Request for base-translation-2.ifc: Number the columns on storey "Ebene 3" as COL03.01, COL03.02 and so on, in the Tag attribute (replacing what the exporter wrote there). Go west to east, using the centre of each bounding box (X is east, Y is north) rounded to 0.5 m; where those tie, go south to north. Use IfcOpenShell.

First a look at what the model holds.

```python
import ifcopenshell
import ifcopenshell.util.element
import ifcopenshell.util.placement

model = ifcopenshell.open("base-translation-2.ifc")
print(model.schema)
storey = next(s for s in model.by_type("IfcBuildingStorey") if s.Name == "Ebene 3")
columns = [e for e in ifcopenshell.util.element.get_decomposition(storey) if e.is_a("IfcColumn")]
for e in sorted(columns, key=lambda e: e.id()):
    origin = ifcopenshell.util.placement.get_local_placement(e.ObjectPlacement)[:3, 3]
    print(e.id(), e.Tag, e.Name, origin.round(2) + 0.0, sep=" | ")
```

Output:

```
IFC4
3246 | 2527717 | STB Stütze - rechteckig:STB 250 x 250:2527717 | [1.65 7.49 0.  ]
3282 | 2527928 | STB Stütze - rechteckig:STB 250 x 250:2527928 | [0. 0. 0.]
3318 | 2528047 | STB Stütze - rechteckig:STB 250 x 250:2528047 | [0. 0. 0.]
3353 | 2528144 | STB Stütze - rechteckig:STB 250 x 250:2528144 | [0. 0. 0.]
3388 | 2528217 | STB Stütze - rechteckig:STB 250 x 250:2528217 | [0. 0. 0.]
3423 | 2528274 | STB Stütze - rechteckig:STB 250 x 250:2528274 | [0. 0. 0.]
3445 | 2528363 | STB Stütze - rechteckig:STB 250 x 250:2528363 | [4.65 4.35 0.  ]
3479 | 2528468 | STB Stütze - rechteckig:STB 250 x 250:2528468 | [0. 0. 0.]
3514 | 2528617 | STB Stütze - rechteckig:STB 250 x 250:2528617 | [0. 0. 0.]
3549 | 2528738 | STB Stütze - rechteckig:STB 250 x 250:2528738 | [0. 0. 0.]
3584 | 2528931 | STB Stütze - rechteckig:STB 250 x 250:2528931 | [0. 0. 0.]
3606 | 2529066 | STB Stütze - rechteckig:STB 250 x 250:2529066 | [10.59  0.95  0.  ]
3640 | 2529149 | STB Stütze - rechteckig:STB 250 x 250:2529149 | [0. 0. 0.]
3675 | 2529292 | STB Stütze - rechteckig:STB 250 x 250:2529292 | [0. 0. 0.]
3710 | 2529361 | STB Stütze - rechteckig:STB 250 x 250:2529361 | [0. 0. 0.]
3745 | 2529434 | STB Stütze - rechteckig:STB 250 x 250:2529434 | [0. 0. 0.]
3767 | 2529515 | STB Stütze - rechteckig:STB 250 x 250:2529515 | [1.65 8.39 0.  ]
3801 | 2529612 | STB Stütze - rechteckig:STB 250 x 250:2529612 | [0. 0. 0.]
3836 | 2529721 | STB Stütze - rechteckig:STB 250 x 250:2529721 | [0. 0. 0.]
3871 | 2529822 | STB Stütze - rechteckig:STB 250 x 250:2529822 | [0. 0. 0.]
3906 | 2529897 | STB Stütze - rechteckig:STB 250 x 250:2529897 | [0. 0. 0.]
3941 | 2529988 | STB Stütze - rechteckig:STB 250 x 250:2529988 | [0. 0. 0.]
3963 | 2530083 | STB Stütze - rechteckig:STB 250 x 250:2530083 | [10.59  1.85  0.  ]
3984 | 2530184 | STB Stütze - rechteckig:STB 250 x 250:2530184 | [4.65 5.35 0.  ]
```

```python
import ifcopenshell
import ifcopenshell.geom
import ifcopenshell.util.element
import ifcopenshell.util.shape

model = ifcopenshell.open("base-translation-2.ifc")
settings = ifcopenshell.geom.settings()
settings.set("use-world-coords", True)


def centre(element):
    shape = ifcopenshell.geom.create_shape(settings, element)
    return ifcopenshell.util.shape.get_bbox_centroid(shape.geometry)


storey = next(s for s in model.by_type("IfcBuildingStorey") if s.Name == "Ebene 3")
columns = [e for e in ifcopenshell.util.element.get_decomposition(storey) if e.is_a("IfcColumn")]

# Insertion points can sit at a corner or the storey origin, so sort by the geometry (in metres).
centres = {e: centre(e) for e in columns}
columns.sort(key=lambda e: (round(centres[e][0] / 0.5), centres[e][1]))

for i, e in enumerate(columns, start=1):
    number = f"COL03.{i:02d}"
    e.Tag = number
    print(e.id(), number)

model.write("base-translation-2_v2.ifc")
```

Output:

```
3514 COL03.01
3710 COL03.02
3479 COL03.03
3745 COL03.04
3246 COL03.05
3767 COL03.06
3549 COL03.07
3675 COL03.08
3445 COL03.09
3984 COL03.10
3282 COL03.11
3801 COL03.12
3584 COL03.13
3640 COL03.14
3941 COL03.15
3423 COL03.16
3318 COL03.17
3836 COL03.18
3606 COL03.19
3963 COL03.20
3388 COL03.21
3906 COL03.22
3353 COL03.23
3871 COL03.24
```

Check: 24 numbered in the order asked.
